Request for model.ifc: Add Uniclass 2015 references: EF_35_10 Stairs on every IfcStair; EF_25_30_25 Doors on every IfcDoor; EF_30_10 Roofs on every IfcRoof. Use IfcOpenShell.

First a look at what the model holds.

```python
import ifcopenshell

model = ifcopenshell.open("model.ifc")
print(model.schema)
print("classifications:", [c.Name for c in model.by_type("IfcClassification")])
for ifc_class in ("IfcDoor", "IfcRoof", "IfcStair", "IfcWall", "IfcWindow"):
    print(ifc_class, len(model.by_type(ifc_class)))
```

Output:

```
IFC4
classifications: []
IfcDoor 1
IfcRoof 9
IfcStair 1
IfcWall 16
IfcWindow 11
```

```python
import ifcopenshell
import ifcopenshell.api.classification

model = ifcopenshell.open("model.ifc")

system = ifcopenshell.api.classification.add_classification(model, classification="Uniclass 2015")

codes = {
    "IfcStair": ("EF_35_10", "Stairs"),
    "IfcDoor": ("EF_25_30_25", "Doors"),
    "IfcRoof": ("EF_30_10", "Roofs"),
}
for ifc_class, (code, name) in codes.items():
    products = model.by_type(ifc_class)
    ifcopenshell.api.classification.add_reference(
        model, products=products, classification=system, identification=code, name=name
    )
    print(code, len(products))

model.write("model_rev.ifc")
```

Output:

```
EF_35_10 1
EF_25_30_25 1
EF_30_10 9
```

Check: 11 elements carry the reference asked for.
